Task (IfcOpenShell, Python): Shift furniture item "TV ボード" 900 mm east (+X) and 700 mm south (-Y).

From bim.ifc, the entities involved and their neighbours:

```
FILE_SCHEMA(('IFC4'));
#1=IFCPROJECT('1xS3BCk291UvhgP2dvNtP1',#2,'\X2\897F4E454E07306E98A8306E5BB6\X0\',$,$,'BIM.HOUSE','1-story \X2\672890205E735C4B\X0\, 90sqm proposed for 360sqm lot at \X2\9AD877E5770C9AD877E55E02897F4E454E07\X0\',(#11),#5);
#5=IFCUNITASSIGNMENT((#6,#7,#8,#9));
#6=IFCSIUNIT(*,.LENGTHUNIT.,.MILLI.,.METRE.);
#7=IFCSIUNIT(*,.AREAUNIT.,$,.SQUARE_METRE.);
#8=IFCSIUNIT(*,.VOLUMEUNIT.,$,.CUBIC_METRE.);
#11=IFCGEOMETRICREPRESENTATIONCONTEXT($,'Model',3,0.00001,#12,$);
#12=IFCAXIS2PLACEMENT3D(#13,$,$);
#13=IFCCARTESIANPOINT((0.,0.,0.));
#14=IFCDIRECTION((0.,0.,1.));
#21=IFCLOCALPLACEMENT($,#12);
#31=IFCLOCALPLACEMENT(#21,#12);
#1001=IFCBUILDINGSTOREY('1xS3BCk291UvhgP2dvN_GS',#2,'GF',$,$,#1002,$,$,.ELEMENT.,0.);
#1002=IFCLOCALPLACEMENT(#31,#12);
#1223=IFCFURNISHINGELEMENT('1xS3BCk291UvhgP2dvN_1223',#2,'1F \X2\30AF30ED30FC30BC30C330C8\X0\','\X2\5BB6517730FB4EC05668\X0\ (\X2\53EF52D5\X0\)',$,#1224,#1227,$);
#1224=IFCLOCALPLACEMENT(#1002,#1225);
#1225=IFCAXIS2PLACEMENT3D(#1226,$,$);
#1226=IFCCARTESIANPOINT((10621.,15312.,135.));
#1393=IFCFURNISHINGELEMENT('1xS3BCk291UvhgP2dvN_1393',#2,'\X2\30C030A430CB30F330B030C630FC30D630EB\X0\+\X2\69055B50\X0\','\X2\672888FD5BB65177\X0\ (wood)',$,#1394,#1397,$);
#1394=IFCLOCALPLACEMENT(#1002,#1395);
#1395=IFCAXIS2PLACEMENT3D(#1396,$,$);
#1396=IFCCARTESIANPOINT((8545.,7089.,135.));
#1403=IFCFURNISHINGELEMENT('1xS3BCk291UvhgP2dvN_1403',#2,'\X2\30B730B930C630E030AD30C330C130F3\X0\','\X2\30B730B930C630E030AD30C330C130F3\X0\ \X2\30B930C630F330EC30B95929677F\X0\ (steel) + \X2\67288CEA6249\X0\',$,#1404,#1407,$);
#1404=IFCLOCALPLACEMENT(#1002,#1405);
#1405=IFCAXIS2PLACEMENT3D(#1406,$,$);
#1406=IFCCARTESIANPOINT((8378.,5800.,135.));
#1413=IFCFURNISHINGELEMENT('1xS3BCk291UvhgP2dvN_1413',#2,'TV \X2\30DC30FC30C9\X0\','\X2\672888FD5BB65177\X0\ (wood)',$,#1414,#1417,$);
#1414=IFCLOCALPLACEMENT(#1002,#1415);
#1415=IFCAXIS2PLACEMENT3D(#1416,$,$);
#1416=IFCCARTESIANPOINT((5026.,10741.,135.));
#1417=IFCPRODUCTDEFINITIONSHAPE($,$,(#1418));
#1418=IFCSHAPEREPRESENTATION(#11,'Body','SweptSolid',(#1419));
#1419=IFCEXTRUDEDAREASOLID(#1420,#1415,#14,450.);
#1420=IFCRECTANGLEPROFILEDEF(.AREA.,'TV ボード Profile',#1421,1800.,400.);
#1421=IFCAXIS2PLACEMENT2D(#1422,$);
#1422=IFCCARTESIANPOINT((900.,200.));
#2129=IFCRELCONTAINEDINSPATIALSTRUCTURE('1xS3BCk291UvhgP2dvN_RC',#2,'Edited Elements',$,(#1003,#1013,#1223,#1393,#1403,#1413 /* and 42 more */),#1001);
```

```python
import ifcopenshell
import ifcopenshell.api.geometry
import ifcopenshell.util.placement

model = ifcopenshell.open("bim.ifc")

item = model.by_guid("1xS3BCk291UvhgP2dvN_1413")
matrix = ifcopenshell.util.placement.get_local_placement(item.ObjectPlacement)
matrix[0, 3] += 900.0
matrix[1, 3] -= 700.0
ifcopenshell.api.geometry.edit_object_placement(model, product=item, matrix=matrix, is_si=False)

print(ifcopenshell.util.placement.get_local_placement(item.ObjectPlacement).round(3) + 0.0)

model.write("bim_updated.ifc")
```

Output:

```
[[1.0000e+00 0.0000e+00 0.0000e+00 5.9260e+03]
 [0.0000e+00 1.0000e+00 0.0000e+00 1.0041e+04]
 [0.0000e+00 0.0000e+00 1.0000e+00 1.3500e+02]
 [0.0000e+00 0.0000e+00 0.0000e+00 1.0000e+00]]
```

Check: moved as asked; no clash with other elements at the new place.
